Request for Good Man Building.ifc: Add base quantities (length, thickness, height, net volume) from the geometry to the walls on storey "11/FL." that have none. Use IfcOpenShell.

First a look at what the model holds.

```python
import ifcopenshell
import ifcopenshell.util.element
import ifcopenshell.util.unit

model = ifcopenshell.open("Good Man Building.ifc")
print(model.schema)
for unit_type in ("LENGTHUNIT", "AREAUNIT", "VOLUMEUNIT"):
    print(unit_type, ifcopenshell.util.unit.calculate_unit_scale(model, unit_type))
storey = next(s for s in model.by_type("IfcBuildingStorey") if s.Name == "11/FL.")
walls = [e for e in ifcopenshell.util.element.get_decomposition(storey) if e.is_a("IfcWall")]
for e in sorted(walls, key=lambda e: e.id()):
    print(e.id(), e.is_a(), e.Name, list(ifcopenshell.util.element.get_psets(e, qtos_only=True)), sep=" | ")
```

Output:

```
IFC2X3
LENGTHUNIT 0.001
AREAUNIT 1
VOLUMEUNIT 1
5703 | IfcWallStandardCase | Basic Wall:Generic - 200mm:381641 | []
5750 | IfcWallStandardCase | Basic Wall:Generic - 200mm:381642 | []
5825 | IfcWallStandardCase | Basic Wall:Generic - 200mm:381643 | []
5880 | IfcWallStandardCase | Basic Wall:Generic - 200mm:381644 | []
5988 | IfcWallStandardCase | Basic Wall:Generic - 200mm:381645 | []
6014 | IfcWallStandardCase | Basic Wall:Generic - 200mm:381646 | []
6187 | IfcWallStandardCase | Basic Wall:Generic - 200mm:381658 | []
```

```python
import ifcopenshell
import ifcopenshell.api.pset
import ifcopenshell.geom
import ifcopenshell.util.element
import ifcopenshell.util.shape
import ifcopenshell.util.unit

model = ifcopenshell.open("Good Man Building.ifc")
unit_scale = ifcopenshell.util.unit.calculate_unit_scale(model)
volume_scale = ifcopenshell.util.unit.calculate_unit_scale(model, "VOLUMEUNIT")
settings = ifcopenshell.geom.settings()

storey = next(s for s in model.by_type("IfcBuildingStorey") if s.Name == "11/FL.")
walls = [e for e in ifcopenshell.util.element.get_decomposition(storey) if e.is_a("IfcWall")]

for e in sorted(walls, key=lambda e: e.id()):
    if ifcopenshell.util.element.get_psets(e, qtos_only=True, should_inherit=False):
        continue
    # Geometry comes back in metres, in the element's own axes.
    shape = ifcopenshell.geom.create_shape(settings, e)
    values = {
        "Length": ifcopenshell.util.shape.get_x(shape.geometry) / unit_scale,
        "Width": ifcopenshell.util.shape.get_y(shape.geometry) / unit_scale,
        "Height": ifcopenshell.util.shape.get_z(shape.geometry) / unit_scale,
        "NetVolume": ifcopenshell.util.shape.get_volume(shape.geometry) / volume_scale,
    }
    qto = ifcopenshell.api.pset.add_qto(model, product=e, name="BaseQuantities")
    ifcopenshell.api.pset.edit_qto(model, qto=qto, properties=values)
    print(e.id(), {k: round(v, 3) for k, v in values.items()})

model.write("Good Man Building_updated.ifc")
```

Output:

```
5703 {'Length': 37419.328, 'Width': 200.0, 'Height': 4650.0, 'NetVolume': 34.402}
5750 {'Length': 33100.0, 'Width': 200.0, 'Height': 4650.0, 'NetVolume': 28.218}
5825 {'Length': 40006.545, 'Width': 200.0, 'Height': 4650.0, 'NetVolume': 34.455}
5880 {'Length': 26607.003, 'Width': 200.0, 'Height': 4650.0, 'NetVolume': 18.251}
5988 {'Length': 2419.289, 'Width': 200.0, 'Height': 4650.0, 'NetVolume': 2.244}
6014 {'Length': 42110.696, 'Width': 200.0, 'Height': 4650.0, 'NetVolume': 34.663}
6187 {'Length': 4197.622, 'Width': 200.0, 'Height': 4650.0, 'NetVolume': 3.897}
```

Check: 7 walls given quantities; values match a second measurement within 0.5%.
